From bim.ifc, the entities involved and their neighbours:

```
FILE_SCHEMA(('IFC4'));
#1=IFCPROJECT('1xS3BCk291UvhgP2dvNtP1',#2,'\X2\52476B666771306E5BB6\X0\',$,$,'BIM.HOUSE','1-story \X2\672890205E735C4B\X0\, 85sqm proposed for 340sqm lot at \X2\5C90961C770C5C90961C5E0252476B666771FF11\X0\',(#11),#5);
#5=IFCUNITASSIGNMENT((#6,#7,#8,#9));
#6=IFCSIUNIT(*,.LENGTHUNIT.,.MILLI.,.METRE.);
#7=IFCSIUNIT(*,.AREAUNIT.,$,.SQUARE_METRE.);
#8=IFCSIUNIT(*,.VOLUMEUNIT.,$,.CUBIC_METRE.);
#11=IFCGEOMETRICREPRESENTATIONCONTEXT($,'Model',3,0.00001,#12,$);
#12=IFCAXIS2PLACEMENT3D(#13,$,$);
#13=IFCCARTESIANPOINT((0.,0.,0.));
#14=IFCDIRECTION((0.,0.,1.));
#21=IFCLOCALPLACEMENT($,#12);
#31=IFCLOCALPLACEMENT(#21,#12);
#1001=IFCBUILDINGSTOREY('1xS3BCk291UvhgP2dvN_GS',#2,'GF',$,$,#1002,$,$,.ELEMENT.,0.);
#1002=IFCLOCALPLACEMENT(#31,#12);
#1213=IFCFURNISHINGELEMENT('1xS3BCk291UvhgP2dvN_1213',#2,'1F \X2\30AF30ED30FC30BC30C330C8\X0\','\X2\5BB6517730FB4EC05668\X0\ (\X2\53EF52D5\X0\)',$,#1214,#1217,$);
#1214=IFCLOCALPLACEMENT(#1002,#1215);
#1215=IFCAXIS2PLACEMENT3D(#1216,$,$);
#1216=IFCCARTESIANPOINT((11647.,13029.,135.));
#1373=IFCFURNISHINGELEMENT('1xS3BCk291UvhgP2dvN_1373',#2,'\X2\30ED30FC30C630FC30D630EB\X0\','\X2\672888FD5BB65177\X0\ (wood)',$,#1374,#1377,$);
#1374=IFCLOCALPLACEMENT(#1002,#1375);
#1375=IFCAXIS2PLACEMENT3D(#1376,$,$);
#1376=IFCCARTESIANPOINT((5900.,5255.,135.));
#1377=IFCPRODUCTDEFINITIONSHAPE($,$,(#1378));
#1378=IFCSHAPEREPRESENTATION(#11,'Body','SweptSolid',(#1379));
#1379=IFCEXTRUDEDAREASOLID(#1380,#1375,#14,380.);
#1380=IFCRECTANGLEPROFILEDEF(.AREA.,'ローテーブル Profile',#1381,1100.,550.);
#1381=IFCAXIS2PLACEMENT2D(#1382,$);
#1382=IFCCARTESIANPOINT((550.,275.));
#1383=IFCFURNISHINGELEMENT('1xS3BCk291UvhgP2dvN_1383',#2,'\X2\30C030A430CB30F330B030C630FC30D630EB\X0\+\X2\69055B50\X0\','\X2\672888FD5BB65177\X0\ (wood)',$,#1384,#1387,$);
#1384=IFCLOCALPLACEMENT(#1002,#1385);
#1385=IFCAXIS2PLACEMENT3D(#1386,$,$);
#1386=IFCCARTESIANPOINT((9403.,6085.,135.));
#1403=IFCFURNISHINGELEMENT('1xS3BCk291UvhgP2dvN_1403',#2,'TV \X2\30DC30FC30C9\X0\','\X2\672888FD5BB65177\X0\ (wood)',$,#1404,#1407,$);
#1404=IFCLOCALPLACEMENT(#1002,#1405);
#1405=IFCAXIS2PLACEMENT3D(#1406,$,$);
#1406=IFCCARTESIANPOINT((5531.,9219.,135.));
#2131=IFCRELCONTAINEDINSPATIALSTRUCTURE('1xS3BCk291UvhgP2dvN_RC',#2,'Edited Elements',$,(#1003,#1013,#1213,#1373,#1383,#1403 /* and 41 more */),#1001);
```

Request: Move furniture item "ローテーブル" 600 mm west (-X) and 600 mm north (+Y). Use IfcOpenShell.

```python
import ifcopenshell
import ifcopenshell.api.geometry
import ifcopenshell.util.placement
import ifcopenshell.util.unit

model = ifcopenshell.open("bim.ifc")
unit_scale = ifcopenshell.util.unit.calculate_unit_scale(model)

item = model.by_guid("1xS3BCk291UvhgP2dvN_1373")
matrix = ifcopenshell.util.placement.get_local_placement(item.ObjectPlacement)
matrix[0, 3] -= 0.6 / unit_scale
matrix[1, 3] += 0.6 / unit_scale
ifcopenshell.api.geometry.edit_object_placement(model, product=item, matrix=matrix, is_si=False)

print(ifcopenshell.util.placement.get_local_placement(item.ObjectPlacement).round(3) + 0.0)

model.write("bim-out.ifc")
```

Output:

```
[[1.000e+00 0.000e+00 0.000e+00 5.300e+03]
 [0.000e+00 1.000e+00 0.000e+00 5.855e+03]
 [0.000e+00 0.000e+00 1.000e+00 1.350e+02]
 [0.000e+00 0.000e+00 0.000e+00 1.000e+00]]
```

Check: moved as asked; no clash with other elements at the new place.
